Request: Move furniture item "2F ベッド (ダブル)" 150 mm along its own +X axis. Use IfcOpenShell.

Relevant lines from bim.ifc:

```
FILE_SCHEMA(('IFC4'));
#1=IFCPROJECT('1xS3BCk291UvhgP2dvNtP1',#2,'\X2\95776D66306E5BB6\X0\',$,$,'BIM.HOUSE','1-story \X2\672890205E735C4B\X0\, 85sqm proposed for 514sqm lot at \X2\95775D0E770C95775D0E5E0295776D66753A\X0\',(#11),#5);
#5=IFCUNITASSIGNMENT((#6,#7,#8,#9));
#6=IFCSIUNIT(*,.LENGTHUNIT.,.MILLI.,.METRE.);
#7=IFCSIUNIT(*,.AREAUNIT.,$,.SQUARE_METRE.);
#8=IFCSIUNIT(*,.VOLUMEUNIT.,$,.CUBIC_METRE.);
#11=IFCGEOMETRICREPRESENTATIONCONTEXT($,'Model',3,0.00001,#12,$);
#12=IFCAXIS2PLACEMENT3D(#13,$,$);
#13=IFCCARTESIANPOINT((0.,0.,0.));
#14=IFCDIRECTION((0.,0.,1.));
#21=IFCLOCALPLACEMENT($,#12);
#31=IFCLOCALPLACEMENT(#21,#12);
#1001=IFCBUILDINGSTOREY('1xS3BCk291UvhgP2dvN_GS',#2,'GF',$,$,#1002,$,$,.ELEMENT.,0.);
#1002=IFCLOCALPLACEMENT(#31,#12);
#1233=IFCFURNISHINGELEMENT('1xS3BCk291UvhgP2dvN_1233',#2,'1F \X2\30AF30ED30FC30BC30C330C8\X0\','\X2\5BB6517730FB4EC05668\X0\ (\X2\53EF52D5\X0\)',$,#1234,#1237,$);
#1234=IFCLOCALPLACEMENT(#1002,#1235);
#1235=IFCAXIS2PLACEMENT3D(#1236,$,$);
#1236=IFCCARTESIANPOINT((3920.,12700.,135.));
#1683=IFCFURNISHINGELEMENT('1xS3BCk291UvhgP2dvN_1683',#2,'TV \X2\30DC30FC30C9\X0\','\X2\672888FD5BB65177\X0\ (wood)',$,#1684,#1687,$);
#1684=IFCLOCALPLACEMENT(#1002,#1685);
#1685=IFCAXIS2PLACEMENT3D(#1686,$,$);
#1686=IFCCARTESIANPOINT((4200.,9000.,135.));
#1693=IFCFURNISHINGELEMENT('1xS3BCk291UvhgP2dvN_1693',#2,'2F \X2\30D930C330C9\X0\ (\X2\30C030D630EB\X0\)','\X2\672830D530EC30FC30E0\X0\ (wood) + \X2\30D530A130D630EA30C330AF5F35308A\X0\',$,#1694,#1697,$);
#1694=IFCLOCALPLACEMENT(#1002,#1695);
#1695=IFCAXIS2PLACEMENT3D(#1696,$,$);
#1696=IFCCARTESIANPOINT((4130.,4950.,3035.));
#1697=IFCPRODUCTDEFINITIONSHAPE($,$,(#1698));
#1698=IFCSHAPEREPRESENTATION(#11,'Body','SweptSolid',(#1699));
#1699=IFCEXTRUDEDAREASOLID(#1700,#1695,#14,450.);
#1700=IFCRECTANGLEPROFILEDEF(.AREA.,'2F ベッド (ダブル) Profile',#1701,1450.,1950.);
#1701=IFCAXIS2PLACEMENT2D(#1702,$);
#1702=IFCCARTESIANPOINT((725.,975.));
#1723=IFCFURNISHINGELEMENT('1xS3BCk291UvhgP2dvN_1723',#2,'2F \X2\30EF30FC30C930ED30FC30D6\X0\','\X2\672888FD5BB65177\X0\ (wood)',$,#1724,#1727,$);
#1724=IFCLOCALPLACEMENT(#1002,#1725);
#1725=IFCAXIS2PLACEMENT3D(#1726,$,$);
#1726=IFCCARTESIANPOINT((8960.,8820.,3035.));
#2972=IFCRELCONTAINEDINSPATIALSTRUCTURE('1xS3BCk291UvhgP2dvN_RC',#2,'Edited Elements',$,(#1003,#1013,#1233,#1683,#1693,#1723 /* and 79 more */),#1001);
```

```python
import ifcopenshell
import ifcopenshell.api.geometry
import ifcopenshell.util.placement
import ifcopenshell.util.unit

model = ifcopenshell.open("bim.ifc")
unit_scale = ifcopenshell.util.unit.calculate_unit_scale(model)

item = model.by_guid("1xS3BCk291UvhgP2dvN_1693")
matrix = ifcopenshell.util.placement.get_local_placement(item.ObjectPlacement)
matrix[:3, 3] += matrix[:3, 0] * 0.15 / unit_scale
ifcopenshell.api.geometry.edit_object_placement(model, product=item, matrix=matrix, is_si=False)

print(ifcopenshell.util.placement.get_local_placement(item.ObjectPlacement).round(3) + 0.0)

model.write("bim_rev.ifc")
```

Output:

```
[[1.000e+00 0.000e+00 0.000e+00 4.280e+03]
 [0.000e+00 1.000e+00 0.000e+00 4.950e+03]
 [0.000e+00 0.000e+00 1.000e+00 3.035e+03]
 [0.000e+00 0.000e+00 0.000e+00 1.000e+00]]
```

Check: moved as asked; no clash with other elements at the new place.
